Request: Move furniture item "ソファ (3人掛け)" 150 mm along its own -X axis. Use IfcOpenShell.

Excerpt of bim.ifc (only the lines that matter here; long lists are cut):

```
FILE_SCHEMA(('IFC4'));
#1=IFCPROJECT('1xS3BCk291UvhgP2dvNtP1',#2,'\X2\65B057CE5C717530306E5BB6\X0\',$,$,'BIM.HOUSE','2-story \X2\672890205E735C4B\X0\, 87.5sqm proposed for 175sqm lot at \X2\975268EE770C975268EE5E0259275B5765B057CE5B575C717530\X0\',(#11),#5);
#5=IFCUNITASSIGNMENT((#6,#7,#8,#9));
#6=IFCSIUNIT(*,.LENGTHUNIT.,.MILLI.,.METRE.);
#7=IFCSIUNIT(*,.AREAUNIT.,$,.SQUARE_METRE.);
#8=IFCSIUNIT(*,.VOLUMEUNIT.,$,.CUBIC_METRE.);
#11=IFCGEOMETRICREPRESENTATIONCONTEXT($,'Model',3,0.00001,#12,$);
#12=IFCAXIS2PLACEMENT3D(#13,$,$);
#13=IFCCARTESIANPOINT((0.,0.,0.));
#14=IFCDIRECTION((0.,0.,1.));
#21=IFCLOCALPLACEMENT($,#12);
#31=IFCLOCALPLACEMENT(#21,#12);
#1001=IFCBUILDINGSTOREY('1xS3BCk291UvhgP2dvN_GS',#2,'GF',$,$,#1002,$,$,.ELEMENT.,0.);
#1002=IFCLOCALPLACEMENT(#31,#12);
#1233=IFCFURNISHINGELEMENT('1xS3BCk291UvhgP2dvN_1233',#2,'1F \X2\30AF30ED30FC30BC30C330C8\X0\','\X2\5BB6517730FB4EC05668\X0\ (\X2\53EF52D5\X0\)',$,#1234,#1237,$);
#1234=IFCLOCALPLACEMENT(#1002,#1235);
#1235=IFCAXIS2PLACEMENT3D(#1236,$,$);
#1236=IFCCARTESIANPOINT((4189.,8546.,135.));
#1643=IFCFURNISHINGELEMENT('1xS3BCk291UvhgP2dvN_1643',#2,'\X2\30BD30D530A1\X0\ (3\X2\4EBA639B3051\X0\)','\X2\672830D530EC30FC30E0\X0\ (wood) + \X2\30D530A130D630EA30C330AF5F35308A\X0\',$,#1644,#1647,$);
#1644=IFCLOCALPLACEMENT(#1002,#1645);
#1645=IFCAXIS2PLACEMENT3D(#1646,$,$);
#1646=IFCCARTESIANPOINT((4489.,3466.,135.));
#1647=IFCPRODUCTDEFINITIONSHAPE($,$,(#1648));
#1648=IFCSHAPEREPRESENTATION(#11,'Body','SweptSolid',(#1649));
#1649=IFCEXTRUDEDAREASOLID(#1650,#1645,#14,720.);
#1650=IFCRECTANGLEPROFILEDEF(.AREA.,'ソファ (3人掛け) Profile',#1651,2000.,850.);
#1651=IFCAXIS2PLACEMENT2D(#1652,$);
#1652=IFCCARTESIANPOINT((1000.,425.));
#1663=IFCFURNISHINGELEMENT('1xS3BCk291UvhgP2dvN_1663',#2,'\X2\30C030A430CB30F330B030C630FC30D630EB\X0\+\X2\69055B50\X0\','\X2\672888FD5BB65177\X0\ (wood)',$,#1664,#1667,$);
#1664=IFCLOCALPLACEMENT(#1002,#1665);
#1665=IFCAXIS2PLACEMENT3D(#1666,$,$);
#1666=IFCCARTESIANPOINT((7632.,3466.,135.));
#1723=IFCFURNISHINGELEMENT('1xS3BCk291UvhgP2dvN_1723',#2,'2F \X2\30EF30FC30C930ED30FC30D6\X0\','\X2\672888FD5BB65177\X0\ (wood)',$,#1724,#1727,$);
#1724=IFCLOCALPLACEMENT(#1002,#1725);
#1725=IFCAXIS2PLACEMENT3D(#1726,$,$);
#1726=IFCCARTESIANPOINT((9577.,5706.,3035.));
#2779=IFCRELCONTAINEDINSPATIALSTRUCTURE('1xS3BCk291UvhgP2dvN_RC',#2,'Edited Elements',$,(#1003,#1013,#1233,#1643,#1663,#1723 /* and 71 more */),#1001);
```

```python
import ifcopenshell
import ifcopenshell.api.geometry
import ifcopenshell.util.placement
import ifcopenshell.util.unit

model = ifcopenshell.open("bim.ifc")
unit_scale = ifcopenshell.util.unit.calculate_unit_scale(model)

item = model.by_id(1643)
matrix = ifcopenshell.util.placement.get_local_placement(item.ObjectPlacement)
matrix[:3, 3] -= matrix[:3, 0] * 0.15 / unit_scale
ifcopenshell.api.geometry.edit_object_placement(model, product=item, matrix=matrix, is_si=False)

print(ifcopenshell.util.placement.get_local_placement(item.ObjectPlacement).round(3) + 0.0)

model.write("bim_v2.ifc")
```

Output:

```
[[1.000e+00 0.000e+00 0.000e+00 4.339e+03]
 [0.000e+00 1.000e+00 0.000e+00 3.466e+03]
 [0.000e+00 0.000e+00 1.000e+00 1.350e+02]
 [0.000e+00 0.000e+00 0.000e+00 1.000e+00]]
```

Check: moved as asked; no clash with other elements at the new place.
